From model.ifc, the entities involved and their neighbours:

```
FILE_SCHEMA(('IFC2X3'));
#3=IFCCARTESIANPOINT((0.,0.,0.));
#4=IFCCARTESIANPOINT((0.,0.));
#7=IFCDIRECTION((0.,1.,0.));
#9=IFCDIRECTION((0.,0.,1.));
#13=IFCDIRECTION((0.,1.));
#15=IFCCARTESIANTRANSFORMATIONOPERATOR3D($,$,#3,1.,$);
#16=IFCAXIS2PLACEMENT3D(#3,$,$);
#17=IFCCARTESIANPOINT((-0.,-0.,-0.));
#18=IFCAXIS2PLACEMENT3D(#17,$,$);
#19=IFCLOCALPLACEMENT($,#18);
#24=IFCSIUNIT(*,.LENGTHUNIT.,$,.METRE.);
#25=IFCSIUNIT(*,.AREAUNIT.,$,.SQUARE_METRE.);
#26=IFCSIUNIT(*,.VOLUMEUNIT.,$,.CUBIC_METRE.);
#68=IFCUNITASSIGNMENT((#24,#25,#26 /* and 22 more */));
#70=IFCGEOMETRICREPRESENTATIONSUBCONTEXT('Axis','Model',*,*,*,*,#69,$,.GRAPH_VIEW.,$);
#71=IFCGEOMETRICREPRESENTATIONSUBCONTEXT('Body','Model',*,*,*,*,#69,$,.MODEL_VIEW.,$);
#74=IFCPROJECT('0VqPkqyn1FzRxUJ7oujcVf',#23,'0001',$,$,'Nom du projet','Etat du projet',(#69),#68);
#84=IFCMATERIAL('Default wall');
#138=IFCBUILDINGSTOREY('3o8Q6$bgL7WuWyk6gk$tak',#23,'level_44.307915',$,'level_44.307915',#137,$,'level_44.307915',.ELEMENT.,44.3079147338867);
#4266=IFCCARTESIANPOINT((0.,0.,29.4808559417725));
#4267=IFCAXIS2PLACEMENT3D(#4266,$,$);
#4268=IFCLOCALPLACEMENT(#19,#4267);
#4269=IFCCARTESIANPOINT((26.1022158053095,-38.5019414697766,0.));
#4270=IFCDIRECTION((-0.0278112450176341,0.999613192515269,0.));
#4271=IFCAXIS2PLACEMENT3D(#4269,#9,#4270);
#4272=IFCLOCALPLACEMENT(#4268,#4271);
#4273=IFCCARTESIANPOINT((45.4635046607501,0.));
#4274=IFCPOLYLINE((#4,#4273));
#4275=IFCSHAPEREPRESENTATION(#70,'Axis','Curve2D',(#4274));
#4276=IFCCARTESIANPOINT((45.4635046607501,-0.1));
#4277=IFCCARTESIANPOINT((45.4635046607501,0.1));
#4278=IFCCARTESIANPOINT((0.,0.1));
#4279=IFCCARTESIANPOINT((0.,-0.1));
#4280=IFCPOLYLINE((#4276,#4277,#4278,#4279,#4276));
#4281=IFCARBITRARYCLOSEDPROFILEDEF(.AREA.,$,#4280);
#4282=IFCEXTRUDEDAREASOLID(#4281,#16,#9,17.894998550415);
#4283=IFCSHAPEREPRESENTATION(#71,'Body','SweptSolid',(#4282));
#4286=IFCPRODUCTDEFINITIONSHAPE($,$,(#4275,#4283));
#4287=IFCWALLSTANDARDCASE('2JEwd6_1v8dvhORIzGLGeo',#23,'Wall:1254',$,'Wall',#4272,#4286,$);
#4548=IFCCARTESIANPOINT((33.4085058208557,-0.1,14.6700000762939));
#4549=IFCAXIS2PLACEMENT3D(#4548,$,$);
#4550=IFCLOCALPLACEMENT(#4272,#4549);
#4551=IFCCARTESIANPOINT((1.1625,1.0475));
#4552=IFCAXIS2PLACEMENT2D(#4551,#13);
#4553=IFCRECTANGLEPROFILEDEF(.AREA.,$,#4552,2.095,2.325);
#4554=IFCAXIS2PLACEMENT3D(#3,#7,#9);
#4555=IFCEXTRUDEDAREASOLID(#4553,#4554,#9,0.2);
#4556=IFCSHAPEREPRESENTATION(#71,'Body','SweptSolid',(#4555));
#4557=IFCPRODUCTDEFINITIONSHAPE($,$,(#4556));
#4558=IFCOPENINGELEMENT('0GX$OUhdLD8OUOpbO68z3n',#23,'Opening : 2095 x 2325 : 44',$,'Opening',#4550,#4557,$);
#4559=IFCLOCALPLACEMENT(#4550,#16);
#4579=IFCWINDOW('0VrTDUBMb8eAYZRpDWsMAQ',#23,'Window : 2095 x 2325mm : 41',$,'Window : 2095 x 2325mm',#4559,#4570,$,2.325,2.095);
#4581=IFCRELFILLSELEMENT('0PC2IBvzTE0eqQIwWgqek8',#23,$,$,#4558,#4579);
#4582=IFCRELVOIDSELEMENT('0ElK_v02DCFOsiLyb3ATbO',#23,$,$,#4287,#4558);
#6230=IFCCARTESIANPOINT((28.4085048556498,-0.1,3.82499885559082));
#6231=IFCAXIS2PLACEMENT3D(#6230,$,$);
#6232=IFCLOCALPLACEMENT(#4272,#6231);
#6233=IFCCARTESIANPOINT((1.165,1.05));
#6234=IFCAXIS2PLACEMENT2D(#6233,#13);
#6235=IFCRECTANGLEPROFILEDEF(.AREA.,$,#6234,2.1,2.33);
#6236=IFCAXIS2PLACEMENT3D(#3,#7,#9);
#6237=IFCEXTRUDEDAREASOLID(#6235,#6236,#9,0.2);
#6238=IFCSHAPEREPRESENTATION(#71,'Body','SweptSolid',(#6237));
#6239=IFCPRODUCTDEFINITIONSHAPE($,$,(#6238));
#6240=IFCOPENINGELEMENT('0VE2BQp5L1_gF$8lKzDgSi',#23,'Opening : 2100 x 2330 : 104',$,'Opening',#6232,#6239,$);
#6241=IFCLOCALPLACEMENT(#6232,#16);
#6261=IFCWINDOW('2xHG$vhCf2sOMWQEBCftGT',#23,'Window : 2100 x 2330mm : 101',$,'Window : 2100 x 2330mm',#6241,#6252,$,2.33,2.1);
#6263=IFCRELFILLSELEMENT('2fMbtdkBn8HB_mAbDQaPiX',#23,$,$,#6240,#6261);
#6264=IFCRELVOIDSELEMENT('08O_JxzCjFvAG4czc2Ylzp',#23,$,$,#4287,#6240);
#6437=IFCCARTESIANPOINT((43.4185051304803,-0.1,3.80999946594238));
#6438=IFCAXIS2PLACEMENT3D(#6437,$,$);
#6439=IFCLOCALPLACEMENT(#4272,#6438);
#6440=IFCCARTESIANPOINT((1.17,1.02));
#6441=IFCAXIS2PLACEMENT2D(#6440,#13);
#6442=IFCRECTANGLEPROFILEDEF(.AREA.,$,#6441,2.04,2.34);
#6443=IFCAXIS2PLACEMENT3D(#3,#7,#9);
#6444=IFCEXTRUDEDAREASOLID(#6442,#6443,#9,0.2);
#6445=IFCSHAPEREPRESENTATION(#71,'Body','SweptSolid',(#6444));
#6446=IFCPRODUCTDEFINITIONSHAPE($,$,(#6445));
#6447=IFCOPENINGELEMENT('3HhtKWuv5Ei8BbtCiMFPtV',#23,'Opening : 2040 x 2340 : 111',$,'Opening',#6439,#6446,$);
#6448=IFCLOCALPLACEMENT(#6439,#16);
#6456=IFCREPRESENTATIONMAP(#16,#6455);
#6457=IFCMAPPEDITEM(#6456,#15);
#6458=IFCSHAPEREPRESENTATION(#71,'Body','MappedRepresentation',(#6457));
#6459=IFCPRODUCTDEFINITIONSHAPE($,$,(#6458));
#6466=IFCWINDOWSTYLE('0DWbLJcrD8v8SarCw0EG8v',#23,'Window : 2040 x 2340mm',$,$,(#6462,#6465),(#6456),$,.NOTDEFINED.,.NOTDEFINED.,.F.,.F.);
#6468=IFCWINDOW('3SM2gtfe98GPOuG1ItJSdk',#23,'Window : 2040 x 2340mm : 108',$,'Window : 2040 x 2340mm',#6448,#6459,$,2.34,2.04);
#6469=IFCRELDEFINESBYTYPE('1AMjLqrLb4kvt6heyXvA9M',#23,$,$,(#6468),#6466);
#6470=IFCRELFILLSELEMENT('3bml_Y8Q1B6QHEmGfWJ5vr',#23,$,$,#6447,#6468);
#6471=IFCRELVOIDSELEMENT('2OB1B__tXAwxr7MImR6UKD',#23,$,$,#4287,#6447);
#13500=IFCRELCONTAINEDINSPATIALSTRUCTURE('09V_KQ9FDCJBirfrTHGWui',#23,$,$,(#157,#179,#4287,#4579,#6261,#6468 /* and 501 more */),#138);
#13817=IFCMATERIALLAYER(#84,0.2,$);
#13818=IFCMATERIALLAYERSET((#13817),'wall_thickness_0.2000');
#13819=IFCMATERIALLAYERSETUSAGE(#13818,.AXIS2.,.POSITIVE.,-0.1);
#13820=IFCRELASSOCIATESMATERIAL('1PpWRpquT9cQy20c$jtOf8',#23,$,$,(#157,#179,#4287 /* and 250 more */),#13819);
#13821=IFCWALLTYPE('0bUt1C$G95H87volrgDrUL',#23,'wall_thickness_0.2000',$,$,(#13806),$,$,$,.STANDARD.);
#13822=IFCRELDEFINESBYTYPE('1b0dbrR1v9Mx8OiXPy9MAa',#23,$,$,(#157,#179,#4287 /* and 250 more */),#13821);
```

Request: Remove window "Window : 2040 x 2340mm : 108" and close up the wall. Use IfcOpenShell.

```python
import ifcopenshell
import ifcopenshell.api.feature
import ifcopenshell.api.root
import ifcopenshell.geom
import ifcopenshell.util.shape

model = ifcopenshell.open("model.ifc")
settings = ifcopenshell.geom.settings()


def volume(element):
    """Net volume in cubic metres, openings subtracted."""
    shape = ifcopenshell.geom.create_shape(settings, element)
    return ifcopenshell.util.shape.get_volume(shape.geometry)


window = model.by_guid("3SM2gtfe98GPOuG1ItJSdk")
opening = window.FillsVoids[0].RelatingOpeningElement
wall = opening.VoidsElements[0].RelatingBuildingElement
before = volume(wall)

ifcopenshell.api.root.remove_product(model, product=window)
ifcopenshell.api.feature.remove_feature(model, feature=opening)

after = volume(wall)

print(f"wall volume {before:.3f} -> {after:.3f} m3")

model.write("model_updated.ifc")
```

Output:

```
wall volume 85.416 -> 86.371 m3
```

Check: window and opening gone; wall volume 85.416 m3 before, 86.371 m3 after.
